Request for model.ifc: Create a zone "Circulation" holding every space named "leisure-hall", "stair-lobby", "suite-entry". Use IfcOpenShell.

First a look at what the model holds.

```python
import ifcopenshell

model = ifcopenshell.open("model.ifc")
print(model.schema)
seen = {}
for space in model.by_type("IfcSpace"):
    seen[space.LongName] = seen.get(space.LongName, 0) + 1
for name, count in sorted(seen.items(), key=str):
    print(count, "x", name)
print("zones:", [z.Name for z in model.by_type("IfcZone")][:20])
```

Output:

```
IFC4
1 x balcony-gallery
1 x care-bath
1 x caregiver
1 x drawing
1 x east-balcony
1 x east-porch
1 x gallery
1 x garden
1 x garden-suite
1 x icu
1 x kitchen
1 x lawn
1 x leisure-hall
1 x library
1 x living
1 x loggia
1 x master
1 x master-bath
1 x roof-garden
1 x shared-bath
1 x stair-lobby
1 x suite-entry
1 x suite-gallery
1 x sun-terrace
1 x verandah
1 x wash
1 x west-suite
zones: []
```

```python
import ifcopenshell
import ifcopenshell.api.group
import ifcopenshell.api.root

model = ifcopenshell.open("model.ifc")

names = {"leisure-hall", "stair-lobby", "suite-entry"}
spaces = [s for s in model.by_type("IfcSpace") if s.LongName in names]

zone = ifcopenshell.api.root.create_entity(model, ifc_class="IfcZone", name="Circulation")
ifcopenshell.api.group.assign_group(model, products=spaces, group=zone)
print(len(spaces), "spaces in", zone.Name)

model.write("model_v2.ifc")
```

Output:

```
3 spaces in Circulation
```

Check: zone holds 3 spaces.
